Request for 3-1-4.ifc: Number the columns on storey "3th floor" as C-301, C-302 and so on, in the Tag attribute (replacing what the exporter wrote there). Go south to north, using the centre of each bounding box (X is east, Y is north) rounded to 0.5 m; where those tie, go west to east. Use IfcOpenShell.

First a look at what the model holds.

```python
import ifcopenshell
import ifcopenshell.util.element
import ifcopenshell.util.placement

model = ifcopenshell.open("3-1-4.ifc")
print(model.schema)
storey = next(s for s in model.by_type("IfcBuildingStorey") if s.Name == "3th floor")
columns = [e for e in ifcopenshell.util.element.get_decomposition(storey) if e.is_a("IfcColumn")]
for e in sorted(columns, key=lambda e: e.id()):
    origin = ifcopenshell.util.placement.get_local_placement(e.ObjectPlacement)[:3, 3]
    print(e.id(), e.Tag, e.Name, origin.round(2) + 0.0, sep=" | ")
```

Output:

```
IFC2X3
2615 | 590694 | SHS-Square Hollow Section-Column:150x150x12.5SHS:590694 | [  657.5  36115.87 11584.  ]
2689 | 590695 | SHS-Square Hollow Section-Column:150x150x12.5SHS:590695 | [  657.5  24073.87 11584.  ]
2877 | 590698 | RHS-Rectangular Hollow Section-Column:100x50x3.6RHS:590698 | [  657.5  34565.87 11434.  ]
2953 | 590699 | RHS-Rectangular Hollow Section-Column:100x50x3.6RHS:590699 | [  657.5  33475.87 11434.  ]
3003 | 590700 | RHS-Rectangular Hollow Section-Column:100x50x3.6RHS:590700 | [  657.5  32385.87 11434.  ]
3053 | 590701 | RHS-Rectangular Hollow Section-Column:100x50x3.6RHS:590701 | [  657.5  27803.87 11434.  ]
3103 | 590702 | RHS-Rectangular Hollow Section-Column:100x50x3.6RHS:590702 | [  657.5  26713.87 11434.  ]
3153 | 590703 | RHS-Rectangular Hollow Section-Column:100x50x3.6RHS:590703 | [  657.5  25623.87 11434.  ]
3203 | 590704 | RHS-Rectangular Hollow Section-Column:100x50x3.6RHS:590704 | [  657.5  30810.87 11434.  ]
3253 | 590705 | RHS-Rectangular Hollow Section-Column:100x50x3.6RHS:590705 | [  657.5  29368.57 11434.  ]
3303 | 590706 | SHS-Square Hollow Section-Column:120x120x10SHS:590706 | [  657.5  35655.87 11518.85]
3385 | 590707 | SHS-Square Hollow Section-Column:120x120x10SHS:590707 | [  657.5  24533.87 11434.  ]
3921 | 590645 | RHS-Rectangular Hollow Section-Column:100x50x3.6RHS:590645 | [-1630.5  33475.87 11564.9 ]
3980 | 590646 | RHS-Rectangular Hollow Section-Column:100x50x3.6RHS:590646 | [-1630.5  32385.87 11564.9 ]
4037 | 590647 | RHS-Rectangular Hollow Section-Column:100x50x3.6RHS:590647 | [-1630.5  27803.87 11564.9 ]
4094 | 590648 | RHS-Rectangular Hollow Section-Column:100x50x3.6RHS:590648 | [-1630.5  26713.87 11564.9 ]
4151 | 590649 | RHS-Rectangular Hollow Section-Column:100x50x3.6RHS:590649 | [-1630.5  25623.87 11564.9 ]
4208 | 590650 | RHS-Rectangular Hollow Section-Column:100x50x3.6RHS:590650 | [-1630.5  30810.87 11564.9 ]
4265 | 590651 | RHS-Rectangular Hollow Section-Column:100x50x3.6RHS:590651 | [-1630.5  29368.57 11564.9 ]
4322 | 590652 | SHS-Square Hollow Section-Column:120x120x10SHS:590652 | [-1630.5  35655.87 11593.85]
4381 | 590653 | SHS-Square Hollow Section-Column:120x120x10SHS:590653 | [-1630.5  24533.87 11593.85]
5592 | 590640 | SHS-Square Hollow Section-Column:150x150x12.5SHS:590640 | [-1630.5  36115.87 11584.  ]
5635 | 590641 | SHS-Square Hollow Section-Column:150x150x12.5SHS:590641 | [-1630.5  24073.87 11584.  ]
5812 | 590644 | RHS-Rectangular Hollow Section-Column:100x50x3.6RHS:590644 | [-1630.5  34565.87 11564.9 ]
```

```python
import ifcopenshell
import ifcopenshell.geom
import ifcopenshell.util.element
import ifcopenshell.util.shape

model = ifcopenshell.open("3-1-4.ifc")
settings = ifcopenshell.geom.settings()
settings.set("use-world-coords", True)


def centre(element):
    shape = ifcopenshell.geom.create_shape(settings, element)
    return ifcopenshell.util.shape.get_bbox_centroid(shape.geometry)


storey = next(s for s in model.by_type("IfcBuildingStorey") if s.Name == "3th floor")
columns = [e for e in ifcopenshell.util.element.get_decomposition(storey) if e.is_a("IfcColumn")]

# Insertion points can sit at a corner or the storey origin, so sort by the geometry (in metres).
centres = {e: centre(e) for e in columns}
columns.sort(key=lambda e: (round(centres[e][1] / 0.5), centres[e][0]))

for i, e in enumerate(columns, start=1):
    number = f"C-3{i:02d}"
    e.Tag = number
    print(e.id(), number)

model.write("3-1-4_edited.ifc")
```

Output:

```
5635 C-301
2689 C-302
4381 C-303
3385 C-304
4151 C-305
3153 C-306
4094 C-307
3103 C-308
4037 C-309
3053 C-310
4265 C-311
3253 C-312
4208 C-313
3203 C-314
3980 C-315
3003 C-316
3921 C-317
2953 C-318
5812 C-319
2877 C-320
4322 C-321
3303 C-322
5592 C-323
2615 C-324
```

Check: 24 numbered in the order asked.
